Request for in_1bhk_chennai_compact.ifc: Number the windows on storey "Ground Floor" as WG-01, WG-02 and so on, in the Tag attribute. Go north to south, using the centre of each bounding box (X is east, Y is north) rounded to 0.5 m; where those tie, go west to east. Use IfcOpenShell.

First a look at what the model holds.

```python
import ifcopenshell
import ifcopenshell.util.element
import ifcopenshell.util.placement

model = ifcopenshell.open("in_1bhk_chennai_compact.ifc")
print(model.schema)
storey = next(s for s in model.by_type("IfcBuildingStorey") if s.Name == "Ground Floor")
windows = [e for e in ifcopenshell.util.element.get_decomposition(storey) if e.is_a("IfcWindow")]
for e in sorted(windows, key=lambda e: e.id()):
    origin = ifcopenshell.util.placement.get_local_placement(e.ObjectPlacement)[:3, 3]
    print(e.id(), e.Tag, e.Name, origin.round(2) + 0.0, sep=" | ")
```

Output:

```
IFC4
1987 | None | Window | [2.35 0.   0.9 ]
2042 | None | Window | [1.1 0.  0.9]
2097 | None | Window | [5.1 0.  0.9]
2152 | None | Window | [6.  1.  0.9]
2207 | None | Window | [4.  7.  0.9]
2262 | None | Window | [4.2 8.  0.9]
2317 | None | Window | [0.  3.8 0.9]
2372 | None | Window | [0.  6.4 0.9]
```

```python
import ifcopenshell
import ifcopenshell.geom
import ifcopenshell.util.element
import ifcopenshell.util.shape

model = ifcopenshell.open("in_1bhk_chennai_compact.ifc")
settings = ifcopenshell.geom.settings()
settings.set("use-world-coords", True)


def centre(element):
    shape = ifcopenshell.geom.create_shape(settings, element)
    return ifcopenshell.util.shape.get_bbox_centroid(shape.geometry)


storey = next(s for s in model.by_type("IfcBuildingStorey") if s.Name == "Ground Floor")
windows = [e for e in ifcopenshell.util.element.get_decomposition(storey) if e.is_a("IfcWindow")]

# Insertion points can sit at a corner or the storey origin, so sort by the geometry (in metres).
centres = {e: centre(e) for e in windows}
windows.sort(key=lambda e: (-round(centres[e][1] / 0.5), centres[e][0]))

for i, e in enumerate(windows, start=1):
    number = f"WG-{i:02d}"
    e.Tag = number
    print(e.id(), number)

model.write("in_1bhk_chennai_compact_edited.ifc")
```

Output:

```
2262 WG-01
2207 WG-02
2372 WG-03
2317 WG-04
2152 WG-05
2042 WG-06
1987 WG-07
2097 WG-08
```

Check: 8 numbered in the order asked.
